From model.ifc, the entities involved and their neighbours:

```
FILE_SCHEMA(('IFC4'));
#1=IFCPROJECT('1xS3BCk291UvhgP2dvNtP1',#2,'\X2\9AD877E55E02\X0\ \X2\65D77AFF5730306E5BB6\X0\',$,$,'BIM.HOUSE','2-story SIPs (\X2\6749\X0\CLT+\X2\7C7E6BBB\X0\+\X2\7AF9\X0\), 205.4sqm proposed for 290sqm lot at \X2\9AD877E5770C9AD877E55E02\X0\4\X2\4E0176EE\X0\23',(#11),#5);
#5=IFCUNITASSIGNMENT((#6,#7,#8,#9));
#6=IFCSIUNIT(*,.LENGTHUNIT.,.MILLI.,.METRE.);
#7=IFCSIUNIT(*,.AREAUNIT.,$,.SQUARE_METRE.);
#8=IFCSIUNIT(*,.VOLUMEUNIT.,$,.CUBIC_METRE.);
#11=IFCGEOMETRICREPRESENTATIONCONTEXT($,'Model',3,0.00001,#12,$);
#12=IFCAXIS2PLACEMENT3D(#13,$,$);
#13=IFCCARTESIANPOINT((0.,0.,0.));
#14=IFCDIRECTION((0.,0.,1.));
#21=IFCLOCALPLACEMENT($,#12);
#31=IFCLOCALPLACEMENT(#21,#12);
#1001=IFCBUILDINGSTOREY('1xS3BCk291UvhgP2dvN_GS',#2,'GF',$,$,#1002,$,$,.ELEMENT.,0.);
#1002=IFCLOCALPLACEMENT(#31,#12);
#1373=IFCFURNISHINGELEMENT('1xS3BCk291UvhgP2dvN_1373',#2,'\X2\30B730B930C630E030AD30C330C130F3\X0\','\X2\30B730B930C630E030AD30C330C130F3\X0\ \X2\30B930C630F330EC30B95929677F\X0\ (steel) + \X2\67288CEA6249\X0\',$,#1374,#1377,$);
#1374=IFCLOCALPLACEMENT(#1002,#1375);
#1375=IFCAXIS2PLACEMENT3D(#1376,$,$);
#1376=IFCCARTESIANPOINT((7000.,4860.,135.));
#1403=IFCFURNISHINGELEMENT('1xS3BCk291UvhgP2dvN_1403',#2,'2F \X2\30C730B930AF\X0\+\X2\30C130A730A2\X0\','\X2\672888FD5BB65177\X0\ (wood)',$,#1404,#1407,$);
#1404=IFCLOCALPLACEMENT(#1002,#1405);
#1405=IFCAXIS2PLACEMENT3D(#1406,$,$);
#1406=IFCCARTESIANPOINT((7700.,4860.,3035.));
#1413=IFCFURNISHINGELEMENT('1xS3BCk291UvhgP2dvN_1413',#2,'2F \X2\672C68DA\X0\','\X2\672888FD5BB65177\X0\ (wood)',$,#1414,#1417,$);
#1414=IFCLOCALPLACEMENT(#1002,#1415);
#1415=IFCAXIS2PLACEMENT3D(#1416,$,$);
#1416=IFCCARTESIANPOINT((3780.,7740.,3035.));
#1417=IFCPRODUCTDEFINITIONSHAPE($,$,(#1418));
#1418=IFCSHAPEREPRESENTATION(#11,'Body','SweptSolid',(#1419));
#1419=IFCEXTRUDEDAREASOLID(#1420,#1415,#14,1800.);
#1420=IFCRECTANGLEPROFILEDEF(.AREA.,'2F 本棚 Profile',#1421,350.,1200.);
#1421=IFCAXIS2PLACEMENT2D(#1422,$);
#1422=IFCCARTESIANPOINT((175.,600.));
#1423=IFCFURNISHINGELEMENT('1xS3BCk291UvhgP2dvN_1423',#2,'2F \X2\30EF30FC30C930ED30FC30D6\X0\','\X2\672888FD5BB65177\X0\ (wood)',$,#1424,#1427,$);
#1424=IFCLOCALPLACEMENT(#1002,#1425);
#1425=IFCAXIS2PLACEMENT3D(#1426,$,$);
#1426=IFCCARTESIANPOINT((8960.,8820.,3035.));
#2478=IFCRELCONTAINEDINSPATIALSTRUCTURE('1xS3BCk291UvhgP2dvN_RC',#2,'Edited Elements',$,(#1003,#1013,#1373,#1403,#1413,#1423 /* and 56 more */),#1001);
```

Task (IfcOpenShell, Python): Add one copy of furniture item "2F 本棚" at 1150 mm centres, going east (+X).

```python
import numpy as np
import ifcopenshell
import ifcopenshell.api.geometry
import ifcopenshell.api.root
import ifcopenshell.util.element
import ifcopenshell.util.placement

model = ifcopenshell.open("model.ifc")


def reuse_history(source, copy):
    """copy_class also copies each property set's owner history, people and application; keep the originals."""
    for rel in copy.IsDefinedBy:
        if rel.is_a("IfcRelDefinesByProperties") and (history := rel.RelatingPropertyDefinition.OwnerHistory):
            rel.RelatingPropertyDefinition.OwnerHistory = source.OwnerHistory
            ifcopenshell.util.element.remove_deep2(model, history)


source = model.by_guid("1xS3BCk291UvhgP2dvN_1413")
base = ifcopenshell.util.placement.get_local_placement(source.ObjectPlacement)
step = np.array([1.0, 0.0, 0.0]) * 1150.0

for i in range(1, 2):
    copy = ifcopenshell.api.root.copy_class(model, product=source)
    copy.Representation = ifcopenshell.util.element.copy_deep(
        model, source.Representation, exclude=["IfcGeometricRepresentationContext", "IfcRepresentationMap"]
    )
    reuse_history(source, copy)
    matrix = base.copy()
    matrix[:3, 3] += i * step
    print("added at", matrix[:3, 3].round(3) + 0.0)
    ifcopenshell.api.geometry.edit_object_placement(model, product=copy, matrix=matrix, is_si=False)

model.write("model-out.ifc")
```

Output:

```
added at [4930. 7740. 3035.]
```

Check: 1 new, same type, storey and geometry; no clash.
